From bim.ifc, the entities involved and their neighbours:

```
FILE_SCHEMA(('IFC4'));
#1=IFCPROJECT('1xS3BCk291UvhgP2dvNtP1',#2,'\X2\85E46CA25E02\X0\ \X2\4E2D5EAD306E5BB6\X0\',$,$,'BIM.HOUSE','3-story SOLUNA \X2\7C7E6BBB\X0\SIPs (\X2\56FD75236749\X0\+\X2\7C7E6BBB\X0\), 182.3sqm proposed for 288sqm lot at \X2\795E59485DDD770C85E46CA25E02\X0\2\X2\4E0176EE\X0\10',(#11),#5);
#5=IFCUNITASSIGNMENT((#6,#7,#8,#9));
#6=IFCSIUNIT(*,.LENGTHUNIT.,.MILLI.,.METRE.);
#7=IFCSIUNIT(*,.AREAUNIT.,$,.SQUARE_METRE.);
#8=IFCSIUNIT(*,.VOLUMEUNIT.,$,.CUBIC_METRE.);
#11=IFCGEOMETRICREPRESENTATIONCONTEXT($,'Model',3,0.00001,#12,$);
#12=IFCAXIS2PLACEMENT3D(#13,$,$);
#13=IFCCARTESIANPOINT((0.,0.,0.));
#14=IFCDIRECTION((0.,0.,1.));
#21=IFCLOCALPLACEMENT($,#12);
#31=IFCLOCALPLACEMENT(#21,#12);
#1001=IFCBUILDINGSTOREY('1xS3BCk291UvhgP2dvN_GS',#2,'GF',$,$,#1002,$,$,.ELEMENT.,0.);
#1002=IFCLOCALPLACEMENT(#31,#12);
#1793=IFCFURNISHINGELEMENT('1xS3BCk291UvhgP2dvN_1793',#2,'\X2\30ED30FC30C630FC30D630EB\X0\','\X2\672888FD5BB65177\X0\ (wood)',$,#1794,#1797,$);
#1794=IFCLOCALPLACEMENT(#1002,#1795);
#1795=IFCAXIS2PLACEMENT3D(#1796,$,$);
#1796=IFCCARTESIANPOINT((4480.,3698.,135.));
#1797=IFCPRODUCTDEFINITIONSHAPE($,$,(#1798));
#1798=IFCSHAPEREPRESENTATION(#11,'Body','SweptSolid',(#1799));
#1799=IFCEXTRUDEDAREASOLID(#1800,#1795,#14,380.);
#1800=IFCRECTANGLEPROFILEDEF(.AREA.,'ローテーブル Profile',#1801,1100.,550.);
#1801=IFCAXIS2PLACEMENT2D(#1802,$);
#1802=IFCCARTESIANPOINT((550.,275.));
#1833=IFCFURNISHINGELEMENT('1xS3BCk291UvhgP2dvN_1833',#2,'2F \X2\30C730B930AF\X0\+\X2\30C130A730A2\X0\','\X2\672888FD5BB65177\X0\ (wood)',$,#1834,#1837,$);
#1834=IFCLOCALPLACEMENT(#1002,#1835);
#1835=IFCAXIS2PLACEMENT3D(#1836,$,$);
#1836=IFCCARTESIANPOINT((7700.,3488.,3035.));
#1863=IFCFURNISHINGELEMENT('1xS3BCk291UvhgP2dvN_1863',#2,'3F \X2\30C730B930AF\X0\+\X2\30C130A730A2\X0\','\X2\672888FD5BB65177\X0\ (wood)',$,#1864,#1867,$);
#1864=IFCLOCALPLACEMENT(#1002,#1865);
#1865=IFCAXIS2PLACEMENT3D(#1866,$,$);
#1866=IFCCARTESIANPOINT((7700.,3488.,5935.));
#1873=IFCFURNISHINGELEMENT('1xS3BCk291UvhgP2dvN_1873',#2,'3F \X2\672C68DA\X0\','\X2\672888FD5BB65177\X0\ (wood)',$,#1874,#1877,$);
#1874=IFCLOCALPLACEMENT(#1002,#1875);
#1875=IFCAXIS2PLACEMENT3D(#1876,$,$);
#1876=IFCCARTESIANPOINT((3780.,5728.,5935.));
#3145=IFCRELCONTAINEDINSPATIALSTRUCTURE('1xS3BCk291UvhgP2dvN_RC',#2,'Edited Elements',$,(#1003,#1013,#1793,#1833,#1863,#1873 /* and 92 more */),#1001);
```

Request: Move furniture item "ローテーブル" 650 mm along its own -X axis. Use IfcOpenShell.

```python
import ifcopenshell
import ifcopenshell.api.geometry
import ifcopenshell.util.placement
import ifcopenshell.util.unit

model = ifcopenshell.open("bim.ifc")
unit_scale = ifcopenshell.util.unit.calculate_unit_scale(model)

item = model.by_guid("1xS3BCk291UvhgP2dvN_1793")
matrix = ifcopenshell.util.placement.get_local_placement(item.ObjectPlacement)
matrix[:3, 3] -= matrix[:3, 0] * 0.65 / unit_scale
ifcopenshell.api.geometry.edit_object_placement(model, product=item, matrix=matrix, is_si=False)

print(ifcopenshell.util.placement.get_local_placement(item.ObjectPlacement).round(3) + 0.0)

model.write("bim_rev.ifc")
```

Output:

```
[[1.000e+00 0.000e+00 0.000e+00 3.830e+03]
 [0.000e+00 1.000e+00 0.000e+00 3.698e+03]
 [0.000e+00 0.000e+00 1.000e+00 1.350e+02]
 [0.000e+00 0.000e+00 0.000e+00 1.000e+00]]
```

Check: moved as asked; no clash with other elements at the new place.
